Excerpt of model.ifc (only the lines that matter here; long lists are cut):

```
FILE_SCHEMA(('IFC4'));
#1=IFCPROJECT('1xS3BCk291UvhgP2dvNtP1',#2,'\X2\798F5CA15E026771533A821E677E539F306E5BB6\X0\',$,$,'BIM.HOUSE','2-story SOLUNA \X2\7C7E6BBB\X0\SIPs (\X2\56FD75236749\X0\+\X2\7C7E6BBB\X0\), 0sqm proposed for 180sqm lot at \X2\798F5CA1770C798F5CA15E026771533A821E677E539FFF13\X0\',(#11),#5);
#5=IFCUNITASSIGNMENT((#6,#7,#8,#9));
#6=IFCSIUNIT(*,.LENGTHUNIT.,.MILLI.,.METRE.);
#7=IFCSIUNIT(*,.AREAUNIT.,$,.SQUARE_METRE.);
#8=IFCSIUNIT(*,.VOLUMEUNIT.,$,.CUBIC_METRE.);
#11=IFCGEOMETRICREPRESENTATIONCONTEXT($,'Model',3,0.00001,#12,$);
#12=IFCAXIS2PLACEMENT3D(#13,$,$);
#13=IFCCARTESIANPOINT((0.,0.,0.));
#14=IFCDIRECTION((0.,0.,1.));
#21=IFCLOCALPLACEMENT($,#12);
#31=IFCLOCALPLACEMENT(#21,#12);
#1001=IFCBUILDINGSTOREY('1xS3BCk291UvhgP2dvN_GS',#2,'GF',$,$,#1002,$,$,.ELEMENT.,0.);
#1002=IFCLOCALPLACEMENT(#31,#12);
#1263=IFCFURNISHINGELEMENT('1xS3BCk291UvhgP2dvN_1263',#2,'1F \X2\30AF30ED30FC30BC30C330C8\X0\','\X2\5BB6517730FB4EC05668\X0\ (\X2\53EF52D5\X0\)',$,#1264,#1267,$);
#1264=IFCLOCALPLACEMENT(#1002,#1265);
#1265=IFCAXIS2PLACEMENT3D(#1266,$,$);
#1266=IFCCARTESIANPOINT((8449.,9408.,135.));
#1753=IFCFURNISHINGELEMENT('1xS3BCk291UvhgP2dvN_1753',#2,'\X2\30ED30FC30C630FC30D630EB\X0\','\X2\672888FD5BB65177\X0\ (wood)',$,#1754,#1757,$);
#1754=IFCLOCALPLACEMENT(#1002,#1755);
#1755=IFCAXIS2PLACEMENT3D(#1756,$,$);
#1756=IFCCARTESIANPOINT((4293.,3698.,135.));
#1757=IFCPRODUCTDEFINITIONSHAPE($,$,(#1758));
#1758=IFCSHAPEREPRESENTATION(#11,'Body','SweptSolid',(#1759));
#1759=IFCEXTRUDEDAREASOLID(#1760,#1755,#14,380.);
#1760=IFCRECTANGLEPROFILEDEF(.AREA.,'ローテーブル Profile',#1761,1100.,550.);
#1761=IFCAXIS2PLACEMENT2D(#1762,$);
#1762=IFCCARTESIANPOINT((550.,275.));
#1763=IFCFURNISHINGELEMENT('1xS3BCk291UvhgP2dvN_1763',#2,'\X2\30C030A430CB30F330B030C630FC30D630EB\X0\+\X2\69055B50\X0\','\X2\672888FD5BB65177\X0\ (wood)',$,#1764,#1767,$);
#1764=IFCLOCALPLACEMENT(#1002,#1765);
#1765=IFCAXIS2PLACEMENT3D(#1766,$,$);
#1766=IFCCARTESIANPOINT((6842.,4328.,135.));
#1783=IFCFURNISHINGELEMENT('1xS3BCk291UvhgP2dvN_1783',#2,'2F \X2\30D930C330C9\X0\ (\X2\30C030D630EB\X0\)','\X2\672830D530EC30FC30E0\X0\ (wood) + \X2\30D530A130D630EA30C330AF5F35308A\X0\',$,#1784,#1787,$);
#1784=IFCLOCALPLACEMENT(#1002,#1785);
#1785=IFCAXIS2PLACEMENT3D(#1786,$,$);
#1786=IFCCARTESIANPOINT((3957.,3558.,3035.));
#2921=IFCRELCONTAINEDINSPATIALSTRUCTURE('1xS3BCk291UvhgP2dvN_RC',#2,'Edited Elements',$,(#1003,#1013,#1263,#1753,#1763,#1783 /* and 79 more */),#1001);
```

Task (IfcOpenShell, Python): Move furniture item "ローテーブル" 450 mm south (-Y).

```python
import ifcopenshell
import ifcopenshell.api.geometry
import ifcopenshell.util.placement

model = ifcopenshell.open("model.ifc")

item = model.by_id(1753)
matrix = ifcopenshell.util.placement.get_local_placement(item.ObjectPlacement)
matrix[1, 3] -= 450.0
ifcopenshell.api.geometry.edit_object_placement(model, product=item, matrix=matrix, is_si=False)

print(ifcopenshell.util.placement.get_local_placement(item.ObjectPlacement).round(3) + 0.0)

model.write("model_edited.ifc")
```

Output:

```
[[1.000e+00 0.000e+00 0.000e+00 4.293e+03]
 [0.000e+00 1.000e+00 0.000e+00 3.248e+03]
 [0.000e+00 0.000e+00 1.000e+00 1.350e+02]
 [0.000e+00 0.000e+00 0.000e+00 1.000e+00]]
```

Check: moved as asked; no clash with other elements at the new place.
